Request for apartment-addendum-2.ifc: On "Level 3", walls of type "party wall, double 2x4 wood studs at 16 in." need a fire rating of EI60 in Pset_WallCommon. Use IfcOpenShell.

First a look at what the model holds.

```python
import ifcopenshell
import ifcopenshell.util.element

model = ifcopenshell.open("apartment-addendum-2.ifc")
print(model.schema)
storey = next(s for s in model.by_type("IfcBuildingStorey") if s.Name == "Level 3")
walls = [e for e in ifcopenshell.util.element.get_decomposition(storey) if e.is_a("IfcWall")]
seen = {}
for e in walls:
    element_type = ifcopenshell.util.element.get_type(e)
    key = (element_type.Name if element_type != e and element_type else None, ifcopenshell.util.element.get_pset(e, "Pset_WallCommon", "FireRating"))
    seen[key] = seen.get(key, 0) + 1
for (name, value), count in sorted(seen.items(), key=str):
    print(count, "x", name, "|", value)
```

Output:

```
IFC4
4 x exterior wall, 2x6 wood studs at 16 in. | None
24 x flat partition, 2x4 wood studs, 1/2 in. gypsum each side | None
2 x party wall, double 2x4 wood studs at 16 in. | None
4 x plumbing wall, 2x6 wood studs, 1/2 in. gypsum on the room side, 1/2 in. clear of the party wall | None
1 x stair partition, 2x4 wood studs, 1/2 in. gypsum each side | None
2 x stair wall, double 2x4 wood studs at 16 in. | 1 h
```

```python
import ifcopenshell
import ifcopenshell.api.pset
import ifcopenshell.util.element

model = ifcopenshell.open("apartment-addendum-2.ifc")

storey = next(s for s in model.by_type("IfcBuildingStorey") if s.Name == "Level 3")
walls = [e for e in ifcopenshell.util.element.get_decomposition(storey) if e.is_a("IfcWall")]

count = 0
for e in walls:
    element_type = ifcopenshell.util.element.get_type(e)
    if element_type in (None, e) or element_type.Name != "party wall, double 2x4 wood studs at 16 in.":
        continue
    # add_pset returns the element's existing set when there is one.
    pset = ifcopenshell.api.pset.add_pset(model, product=e, name="Pset_WallCommon")
    ifcopenshell.api.pset.edit_pset(model, pset=pset, properties={"FireRating": "EI60"})
    count += 1

print(count, "walls updated")

model.write("apartment-addendum-2_updated.ifc")
```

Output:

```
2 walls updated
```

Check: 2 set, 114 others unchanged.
